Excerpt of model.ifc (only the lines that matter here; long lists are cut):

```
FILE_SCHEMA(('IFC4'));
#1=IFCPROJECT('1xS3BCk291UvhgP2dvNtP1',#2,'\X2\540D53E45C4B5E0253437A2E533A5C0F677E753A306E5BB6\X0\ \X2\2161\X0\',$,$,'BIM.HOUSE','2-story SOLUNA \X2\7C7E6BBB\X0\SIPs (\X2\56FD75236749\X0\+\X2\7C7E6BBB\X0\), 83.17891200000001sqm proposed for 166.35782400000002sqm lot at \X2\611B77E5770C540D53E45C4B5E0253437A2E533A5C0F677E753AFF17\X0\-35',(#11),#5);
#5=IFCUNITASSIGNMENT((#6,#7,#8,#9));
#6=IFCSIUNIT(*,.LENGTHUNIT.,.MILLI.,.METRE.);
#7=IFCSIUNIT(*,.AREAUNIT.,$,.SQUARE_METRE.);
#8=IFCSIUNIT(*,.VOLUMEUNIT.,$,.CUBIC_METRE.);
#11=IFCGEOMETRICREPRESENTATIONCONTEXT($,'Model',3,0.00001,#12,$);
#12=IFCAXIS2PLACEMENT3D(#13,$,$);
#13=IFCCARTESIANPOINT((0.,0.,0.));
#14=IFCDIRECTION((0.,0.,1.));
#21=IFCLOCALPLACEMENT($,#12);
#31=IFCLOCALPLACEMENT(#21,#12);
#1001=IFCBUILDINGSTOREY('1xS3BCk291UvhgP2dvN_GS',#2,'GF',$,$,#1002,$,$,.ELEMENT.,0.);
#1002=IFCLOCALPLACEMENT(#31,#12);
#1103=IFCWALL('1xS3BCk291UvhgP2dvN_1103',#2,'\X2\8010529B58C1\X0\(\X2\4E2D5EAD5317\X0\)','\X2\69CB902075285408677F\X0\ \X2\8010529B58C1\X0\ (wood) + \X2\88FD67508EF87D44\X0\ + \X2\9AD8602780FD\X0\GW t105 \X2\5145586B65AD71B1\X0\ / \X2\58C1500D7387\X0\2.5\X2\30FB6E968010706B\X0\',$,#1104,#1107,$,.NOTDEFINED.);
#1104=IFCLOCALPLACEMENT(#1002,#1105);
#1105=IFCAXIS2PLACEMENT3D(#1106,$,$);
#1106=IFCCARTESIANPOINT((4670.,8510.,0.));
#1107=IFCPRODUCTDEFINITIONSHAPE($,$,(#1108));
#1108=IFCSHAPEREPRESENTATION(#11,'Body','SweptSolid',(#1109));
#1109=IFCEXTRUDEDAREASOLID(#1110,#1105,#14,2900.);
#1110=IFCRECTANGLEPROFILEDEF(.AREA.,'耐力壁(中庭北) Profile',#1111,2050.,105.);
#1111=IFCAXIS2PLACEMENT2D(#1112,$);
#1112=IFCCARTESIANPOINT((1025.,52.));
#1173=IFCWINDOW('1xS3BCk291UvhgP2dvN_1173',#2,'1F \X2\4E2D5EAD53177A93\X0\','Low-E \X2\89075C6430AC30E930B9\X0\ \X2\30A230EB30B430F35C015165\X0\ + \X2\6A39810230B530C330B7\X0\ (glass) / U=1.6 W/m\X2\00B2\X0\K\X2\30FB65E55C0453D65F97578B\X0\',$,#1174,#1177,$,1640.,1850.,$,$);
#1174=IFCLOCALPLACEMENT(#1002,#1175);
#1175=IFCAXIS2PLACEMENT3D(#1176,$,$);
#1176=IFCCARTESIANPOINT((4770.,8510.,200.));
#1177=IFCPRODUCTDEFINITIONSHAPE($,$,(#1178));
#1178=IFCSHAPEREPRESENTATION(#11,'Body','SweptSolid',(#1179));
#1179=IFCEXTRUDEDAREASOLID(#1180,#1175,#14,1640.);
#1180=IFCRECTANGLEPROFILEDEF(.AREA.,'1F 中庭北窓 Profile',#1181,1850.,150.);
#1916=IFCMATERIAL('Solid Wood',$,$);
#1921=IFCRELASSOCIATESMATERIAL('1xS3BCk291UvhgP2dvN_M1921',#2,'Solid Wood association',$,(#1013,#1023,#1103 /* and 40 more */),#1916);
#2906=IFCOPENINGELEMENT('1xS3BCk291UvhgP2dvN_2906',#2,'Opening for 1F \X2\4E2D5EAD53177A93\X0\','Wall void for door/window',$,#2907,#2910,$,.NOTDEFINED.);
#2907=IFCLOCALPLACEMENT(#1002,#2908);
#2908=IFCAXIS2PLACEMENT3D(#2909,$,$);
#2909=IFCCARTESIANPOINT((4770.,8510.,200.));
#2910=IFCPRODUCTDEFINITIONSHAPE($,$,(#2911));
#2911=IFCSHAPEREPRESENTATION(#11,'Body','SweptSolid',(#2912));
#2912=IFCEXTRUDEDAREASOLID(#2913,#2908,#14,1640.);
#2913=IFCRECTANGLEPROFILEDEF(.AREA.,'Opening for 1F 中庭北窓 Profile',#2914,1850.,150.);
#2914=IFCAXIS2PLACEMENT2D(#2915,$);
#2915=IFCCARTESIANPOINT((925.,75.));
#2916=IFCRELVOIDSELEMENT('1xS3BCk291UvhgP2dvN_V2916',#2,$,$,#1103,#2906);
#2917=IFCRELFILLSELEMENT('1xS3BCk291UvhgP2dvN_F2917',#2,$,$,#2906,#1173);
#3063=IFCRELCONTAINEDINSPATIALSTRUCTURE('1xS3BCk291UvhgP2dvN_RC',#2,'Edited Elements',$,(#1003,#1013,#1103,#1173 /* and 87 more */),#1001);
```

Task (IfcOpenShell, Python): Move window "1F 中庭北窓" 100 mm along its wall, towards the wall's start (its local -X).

```python
import ifcopenshell
import ifcopenshell.api.geometry
import ifcopenshell.util.placement

model = ifcopenshell.open("model.ifc")

window = model.by_guid("1xS3BCk291UvhgP2dvN_1173")
opening = window.FillsVoids[0].RelatingOpeningElement
wall = opening.VoidsElements[0].RelatingBuildingElement

wall_matrix = ifcopenshell.util.placement.get_local_placement(wall.ObjectPlacement)
shift = wall_matrix[:3, 0] * -100.0
before = ifcopenshell.util.placement.get_local_placement(window.ObjectPlacement)[:3, 3].copy()

# The window is not placed relative to its opening, so move both.
for product in (opening, window):
    matrix = ifcopenshell.util.placement.get_local_placement(product.ObjectPlacement)
    matrix[:3, 3] += shift
    ifcopenshell.api.geometry.edit_object_placement(model, product=product, matrix=matrix, is_si=False)

after = ifcopenshell.util.placement.get_local_placement(window.ObjectPlacement)[:3, 3]
print("window moved by", (after - before).round(3) + 0.0)

model.write("model_rev.ifc")
```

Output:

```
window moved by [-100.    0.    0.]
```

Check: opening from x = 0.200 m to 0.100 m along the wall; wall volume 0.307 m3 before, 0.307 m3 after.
